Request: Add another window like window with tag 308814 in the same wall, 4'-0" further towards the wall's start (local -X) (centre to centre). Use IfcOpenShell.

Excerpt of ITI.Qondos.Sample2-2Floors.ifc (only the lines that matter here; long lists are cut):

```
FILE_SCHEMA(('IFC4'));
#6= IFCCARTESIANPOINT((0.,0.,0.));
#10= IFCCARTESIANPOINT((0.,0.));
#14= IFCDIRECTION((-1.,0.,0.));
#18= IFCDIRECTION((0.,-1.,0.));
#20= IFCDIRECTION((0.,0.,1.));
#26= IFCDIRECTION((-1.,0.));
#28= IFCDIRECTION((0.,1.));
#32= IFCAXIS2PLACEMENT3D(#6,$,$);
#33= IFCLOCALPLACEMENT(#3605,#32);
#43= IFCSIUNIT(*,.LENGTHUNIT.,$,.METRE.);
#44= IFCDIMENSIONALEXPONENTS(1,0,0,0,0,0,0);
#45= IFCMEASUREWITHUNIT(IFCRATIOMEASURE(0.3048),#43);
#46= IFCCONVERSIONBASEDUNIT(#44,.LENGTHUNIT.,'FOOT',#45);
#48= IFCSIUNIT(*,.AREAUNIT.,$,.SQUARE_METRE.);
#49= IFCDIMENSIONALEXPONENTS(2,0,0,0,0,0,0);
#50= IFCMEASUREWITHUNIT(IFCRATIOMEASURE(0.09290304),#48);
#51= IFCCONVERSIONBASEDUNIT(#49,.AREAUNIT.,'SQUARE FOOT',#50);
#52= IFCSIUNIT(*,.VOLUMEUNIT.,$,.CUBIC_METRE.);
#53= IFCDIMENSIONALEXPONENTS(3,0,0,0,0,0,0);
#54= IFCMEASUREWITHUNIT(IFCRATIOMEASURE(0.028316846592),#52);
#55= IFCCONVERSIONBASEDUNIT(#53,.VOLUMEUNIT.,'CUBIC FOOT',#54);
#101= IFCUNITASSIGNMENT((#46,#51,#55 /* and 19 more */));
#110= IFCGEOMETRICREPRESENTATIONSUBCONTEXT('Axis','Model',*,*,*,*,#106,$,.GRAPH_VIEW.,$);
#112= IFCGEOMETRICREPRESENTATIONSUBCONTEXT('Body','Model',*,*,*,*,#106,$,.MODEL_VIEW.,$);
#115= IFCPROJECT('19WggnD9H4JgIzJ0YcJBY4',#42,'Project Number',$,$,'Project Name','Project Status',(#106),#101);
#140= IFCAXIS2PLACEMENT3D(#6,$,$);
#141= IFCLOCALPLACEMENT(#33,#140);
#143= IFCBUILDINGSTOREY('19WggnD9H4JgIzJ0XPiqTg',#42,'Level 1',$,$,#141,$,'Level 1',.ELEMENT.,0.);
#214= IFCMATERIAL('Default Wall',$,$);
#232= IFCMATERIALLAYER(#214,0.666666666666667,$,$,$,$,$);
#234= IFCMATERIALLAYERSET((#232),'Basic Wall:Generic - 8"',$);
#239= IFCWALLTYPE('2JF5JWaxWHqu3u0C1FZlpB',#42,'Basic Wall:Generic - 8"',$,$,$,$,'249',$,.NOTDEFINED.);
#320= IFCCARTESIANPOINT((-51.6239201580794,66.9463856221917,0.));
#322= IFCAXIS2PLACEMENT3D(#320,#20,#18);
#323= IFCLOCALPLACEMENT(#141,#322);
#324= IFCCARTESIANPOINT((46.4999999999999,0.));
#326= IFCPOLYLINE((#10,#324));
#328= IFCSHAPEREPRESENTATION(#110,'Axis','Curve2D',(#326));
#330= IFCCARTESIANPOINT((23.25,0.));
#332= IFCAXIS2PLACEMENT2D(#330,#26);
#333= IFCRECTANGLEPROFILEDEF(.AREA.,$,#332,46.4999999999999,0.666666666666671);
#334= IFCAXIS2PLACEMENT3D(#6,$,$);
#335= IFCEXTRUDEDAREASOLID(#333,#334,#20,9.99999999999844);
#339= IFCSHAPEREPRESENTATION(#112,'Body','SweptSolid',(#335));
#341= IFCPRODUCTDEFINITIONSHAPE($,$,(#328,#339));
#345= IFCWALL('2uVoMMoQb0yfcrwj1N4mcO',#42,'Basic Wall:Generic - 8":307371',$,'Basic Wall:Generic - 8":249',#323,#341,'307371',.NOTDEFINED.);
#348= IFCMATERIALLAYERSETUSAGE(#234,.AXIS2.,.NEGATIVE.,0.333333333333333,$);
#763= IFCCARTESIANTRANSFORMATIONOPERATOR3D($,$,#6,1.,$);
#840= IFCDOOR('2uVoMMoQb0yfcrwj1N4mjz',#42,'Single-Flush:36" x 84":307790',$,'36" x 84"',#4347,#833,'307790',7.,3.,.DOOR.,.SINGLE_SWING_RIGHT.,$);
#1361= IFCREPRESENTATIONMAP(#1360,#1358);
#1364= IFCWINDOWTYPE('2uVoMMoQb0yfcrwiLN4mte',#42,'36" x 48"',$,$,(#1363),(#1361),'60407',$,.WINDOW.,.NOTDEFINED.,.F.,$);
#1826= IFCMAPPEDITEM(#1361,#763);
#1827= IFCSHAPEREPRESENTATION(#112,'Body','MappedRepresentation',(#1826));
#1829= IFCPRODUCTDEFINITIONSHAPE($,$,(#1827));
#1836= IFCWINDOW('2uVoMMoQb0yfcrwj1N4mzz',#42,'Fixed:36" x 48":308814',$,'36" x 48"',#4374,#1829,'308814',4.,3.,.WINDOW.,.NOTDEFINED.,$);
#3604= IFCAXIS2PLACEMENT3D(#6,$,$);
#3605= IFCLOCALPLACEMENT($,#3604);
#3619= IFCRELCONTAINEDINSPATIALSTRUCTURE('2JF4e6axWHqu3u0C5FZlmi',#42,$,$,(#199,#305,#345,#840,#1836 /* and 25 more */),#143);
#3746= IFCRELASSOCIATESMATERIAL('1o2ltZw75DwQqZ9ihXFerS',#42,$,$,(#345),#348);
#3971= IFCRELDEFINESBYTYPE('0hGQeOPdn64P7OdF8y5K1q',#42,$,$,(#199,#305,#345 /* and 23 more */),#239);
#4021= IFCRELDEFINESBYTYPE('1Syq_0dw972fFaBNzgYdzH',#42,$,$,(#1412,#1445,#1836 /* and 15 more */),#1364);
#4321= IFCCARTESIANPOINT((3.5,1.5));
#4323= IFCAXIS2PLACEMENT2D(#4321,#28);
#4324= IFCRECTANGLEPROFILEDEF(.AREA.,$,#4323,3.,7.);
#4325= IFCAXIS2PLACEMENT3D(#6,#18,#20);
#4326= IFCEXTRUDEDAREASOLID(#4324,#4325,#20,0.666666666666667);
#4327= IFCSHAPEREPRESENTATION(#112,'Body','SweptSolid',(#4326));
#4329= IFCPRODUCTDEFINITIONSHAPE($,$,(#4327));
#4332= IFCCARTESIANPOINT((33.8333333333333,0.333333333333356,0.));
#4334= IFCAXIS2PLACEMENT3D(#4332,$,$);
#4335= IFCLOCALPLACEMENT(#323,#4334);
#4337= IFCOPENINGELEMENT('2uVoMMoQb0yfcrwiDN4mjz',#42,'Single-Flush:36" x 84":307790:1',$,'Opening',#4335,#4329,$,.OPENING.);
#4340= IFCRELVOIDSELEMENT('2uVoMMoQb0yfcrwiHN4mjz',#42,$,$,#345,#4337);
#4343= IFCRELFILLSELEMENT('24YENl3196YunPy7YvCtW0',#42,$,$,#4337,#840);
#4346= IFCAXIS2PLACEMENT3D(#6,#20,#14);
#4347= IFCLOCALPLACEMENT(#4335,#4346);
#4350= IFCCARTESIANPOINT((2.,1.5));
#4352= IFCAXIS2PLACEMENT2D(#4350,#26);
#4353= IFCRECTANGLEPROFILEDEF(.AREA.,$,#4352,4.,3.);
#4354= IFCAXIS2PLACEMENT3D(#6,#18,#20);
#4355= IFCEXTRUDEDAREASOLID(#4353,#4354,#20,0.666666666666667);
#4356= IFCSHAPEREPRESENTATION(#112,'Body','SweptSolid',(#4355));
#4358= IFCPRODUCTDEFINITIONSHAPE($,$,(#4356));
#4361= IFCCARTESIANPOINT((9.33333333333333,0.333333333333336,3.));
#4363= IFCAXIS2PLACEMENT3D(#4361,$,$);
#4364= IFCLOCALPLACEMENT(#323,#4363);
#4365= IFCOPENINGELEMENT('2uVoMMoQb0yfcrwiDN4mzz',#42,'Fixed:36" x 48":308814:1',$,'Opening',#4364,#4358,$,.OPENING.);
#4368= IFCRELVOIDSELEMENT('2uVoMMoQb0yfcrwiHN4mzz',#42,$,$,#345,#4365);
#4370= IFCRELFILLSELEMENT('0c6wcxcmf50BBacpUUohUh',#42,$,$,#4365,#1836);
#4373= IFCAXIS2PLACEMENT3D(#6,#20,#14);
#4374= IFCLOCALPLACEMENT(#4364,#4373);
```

```python
import ifcopenshell
import ifcopenshell.api.feature
import ifcopenshell.api.geometry
import ifcopenshell.api.root
import ifcopenshell.geom
import ifcopenshell.util.element
import ifcopenshell.util.placement
import ifcopenshell.util.shape
import ifcopenshell.util.unit

model = ifcopenshell.open("ITI.Qondos.Sample2-2Floors.ifc")
unit_scale = ifcopenshell.util.unit.calculate_unit_scale(model)
settings = ifcopenshell.geom.settings()


def volume(element):
    """Net volume in cubic metres, openings subtracted."""
    shape = ifcopenshell.geom.create_shape(settings, element)
    return ifcopenshell.util.shape.get_volume(shape.geometry)


def reuse_history(source, copy):
    """copy_class also copies each property set's owner history, people and application; keep the originals."""
    for rel in copy.IsDefinedBy:
        if rel.is_a("IfcRelDefinesByProperties") and (history := rel.RelatingPropertyDefinition.OwnerHistory):
            rel.RelatingPropertyDefinition.OwnerHistory = source.OwnerHistory
            ifcopenshell.util.element.remove_deep2(model, history)


window = model.by_guid("2uVoMMoQb0yfcrwj1N4mzz")
opening = window.FillsVoids[0].RelatingOpeningElement
wall = opening.VoidsElements[0].RelatingBuildingElement
before = volume(wall)
shift = ifcopenshell.util.placement.get_local_placement(wall.ObjectPlacement)[:3, 0] * -48 * 0.0254 / unit_scale

# copy_class copies the void relationship, type, container and properties, but no geometry.
new_opening = ifcopenshell.api.root.copy_class(model, product=opening)
new_opening.Representation = ifcopenshell.util.element.copy_deep(
    model, opening.Representation, exclude=["IfcGeometricRepresentationContext", "IfcRepresentationMap"]
)
new_opening.Name = 'Fixed:36" x 48"'
new_window = ifcopenshell.api.root.copy_class(model, product=window)
new_window.Representation = ifcopenshell.util.element.copy_deep(
    model, window.Representation, exclude=["IfcGeometricRepresentationContext", "IfcRepresentationMap"]
)
new_window.Name = 'Fixed:36" x 48"'
new_window.Tag = None
reuse_history(window, new_window)
ifcopenshell.api.feature.add_filling(model, opening=new_opening, element=new_window)

for old, new in ((opening, new_opening), (window, new_window)):
    matrix = ifcopenshell.util.placement.get_local_placement(old.ObjectPlacement)
    matrix[:3, 3] += shift
    ifcopenshell.api.geometry.edit_object_placement(model, product=new, matrix=matrix, is_si=False)

after = volume(wall)

print(f"wall volume {before:.3f} -> {after:.3f} m3")

model.write("ITI.Qondos.Sample2-2Floors_edited.ifc")
```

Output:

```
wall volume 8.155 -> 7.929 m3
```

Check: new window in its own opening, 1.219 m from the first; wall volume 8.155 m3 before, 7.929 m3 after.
